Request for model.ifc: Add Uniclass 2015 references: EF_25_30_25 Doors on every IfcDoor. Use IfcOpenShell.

First a look at what the model holds.

```python
import ifcopenshell

model = ifcopenshell.open("model.ifc")
print(model.schema)
print("classifications:", [c.Name for c in model.by_type("IfcClassification")])
for ifc_class in ("IfcDoor", "IfcRoof", "IfcStair", "IfcWall", "IfcWindow"):
    print(ifc_class, len(model.by_type(ifc_class)))
```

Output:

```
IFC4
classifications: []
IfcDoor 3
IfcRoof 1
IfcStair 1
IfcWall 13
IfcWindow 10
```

```python
import ifcopenshell
import ifcopenshell.api.classification

model = ifcopenshell.open("model.ifc")

system = ifcopenshell.api.classification.add_classification(model, classification="Uniclass 2015")

codes = {
    "IfcDoor": ("EF_25_30_25", "Doors"),
}
for ifc_class, (code, name) in codes.items():
    products = model.by_type(ifc_class)
    ifcopenshell.api.classification.add_reference(
        model, products=products, classification=system, identification=code, name=name
    )
    print(code, len(products))

model.write("model_updated.ifc")
```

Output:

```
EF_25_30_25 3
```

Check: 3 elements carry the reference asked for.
